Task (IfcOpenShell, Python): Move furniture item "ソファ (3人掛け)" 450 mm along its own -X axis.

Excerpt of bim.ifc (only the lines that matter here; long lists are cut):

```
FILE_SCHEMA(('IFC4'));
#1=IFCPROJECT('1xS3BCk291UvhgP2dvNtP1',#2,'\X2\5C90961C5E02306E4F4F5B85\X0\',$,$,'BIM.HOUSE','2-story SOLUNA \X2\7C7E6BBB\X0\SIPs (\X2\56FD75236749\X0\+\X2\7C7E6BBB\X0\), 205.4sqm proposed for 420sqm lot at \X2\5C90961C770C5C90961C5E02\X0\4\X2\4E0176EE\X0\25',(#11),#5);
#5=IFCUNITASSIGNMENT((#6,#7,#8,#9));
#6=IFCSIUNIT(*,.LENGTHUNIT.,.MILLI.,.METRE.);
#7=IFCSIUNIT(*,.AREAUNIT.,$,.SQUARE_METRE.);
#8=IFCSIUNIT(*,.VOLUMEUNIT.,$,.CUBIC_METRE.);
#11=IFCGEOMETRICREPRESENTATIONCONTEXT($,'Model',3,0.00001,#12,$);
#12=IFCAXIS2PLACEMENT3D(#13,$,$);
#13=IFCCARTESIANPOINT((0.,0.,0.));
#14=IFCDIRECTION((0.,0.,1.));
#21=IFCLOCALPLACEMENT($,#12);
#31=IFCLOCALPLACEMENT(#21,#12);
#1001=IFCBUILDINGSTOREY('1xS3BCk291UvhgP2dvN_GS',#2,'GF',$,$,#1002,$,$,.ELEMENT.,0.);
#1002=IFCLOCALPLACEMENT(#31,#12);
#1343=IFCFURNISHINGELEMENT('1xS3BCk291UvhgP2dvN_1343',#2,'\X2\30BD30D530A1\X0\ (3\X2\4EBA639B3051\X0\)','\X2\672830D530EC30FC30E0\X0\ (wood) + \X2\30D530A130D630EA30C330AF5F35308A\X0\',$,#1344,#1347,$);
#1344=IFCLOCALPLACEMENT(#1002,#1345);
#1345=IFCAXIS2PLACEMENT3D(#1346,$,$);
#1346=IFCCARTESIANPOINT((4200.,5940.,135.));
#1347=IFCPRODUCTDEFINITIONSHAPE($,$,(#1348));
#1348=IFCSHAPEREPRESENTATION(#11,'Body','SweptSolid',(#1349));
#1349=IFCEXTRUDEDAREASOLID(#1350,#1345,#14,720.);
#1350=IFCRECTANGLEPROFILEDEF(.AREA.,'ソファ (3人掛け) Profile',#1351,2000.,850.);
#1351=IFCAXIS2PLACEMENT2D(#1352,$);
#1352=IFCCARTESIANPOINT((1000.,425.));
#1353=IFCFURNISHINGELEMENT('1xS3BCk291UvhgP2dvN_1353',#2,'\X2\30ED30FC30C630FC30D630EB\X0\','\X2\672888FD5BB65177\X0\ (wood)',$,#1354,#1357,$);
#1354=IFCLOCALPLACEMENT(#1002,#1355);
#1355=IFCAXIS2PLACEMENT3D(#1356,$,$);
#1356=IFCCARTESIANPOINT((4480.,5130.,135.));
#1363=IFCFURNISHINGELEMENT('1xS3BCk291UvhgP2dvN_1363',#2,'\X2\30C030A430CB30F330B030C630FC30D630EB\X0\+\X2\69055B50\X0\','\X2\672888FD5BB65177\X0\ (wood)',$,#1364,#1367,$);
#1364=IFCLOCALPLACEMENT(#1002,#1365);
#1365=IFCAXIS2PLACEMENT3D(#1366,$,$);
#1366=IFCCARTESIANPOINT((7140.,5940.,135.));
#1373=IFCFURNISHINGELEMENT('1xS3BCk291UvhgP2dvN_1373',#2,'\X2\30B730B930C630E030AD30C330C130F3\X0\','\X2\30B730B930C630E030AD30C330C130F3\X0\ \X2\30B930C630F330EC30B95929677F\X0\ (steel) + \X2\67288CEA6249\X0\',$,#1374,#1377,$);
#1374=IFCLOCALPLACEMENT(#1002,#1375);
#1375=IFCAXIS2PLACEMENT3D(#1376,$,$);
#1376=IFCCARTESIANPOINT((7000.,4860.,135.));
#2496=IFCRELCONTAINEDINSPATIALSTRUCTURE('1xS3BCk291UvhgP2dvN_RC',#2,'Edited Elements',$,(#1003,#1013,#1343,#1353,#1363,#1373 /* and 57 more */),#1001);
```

```python
import ifcopenshell
import ifcopenshell.api.geometry
import ifcopenshell.util.placement
import ifcopenshell.util.unit

model = ifcopenshell.open("bim.ifc")
unit_scale = ifcopenshell.util.unit.calculate_unit_scale(model)

item = model.by_guid("1xS3BCk291UvhgP2dvN_1343")
matrix = ifcopenshell.util.placement.get_local_placement(item.ObjectPlacement)
matrix[:3, 3] -= matrix[:3, 0] * 0.45 / unit_scale
ifcopenshell.api.geometry.edit_object_placement(model, product=item, matrix=matrix, is_si=False)

print(ifcopenshell.util.placement.get_local_placement(item.ObjectPlacement).round(3) + 0.0)

model.write("bim-out.ifc")
```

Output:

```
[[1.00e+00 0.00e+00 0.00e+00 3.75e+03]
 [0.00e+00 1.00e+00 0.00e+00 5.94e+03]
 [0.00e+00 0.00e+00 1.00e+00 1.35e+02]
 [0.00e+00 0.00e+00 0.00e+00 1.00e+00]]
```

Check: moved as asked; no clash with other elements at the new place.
